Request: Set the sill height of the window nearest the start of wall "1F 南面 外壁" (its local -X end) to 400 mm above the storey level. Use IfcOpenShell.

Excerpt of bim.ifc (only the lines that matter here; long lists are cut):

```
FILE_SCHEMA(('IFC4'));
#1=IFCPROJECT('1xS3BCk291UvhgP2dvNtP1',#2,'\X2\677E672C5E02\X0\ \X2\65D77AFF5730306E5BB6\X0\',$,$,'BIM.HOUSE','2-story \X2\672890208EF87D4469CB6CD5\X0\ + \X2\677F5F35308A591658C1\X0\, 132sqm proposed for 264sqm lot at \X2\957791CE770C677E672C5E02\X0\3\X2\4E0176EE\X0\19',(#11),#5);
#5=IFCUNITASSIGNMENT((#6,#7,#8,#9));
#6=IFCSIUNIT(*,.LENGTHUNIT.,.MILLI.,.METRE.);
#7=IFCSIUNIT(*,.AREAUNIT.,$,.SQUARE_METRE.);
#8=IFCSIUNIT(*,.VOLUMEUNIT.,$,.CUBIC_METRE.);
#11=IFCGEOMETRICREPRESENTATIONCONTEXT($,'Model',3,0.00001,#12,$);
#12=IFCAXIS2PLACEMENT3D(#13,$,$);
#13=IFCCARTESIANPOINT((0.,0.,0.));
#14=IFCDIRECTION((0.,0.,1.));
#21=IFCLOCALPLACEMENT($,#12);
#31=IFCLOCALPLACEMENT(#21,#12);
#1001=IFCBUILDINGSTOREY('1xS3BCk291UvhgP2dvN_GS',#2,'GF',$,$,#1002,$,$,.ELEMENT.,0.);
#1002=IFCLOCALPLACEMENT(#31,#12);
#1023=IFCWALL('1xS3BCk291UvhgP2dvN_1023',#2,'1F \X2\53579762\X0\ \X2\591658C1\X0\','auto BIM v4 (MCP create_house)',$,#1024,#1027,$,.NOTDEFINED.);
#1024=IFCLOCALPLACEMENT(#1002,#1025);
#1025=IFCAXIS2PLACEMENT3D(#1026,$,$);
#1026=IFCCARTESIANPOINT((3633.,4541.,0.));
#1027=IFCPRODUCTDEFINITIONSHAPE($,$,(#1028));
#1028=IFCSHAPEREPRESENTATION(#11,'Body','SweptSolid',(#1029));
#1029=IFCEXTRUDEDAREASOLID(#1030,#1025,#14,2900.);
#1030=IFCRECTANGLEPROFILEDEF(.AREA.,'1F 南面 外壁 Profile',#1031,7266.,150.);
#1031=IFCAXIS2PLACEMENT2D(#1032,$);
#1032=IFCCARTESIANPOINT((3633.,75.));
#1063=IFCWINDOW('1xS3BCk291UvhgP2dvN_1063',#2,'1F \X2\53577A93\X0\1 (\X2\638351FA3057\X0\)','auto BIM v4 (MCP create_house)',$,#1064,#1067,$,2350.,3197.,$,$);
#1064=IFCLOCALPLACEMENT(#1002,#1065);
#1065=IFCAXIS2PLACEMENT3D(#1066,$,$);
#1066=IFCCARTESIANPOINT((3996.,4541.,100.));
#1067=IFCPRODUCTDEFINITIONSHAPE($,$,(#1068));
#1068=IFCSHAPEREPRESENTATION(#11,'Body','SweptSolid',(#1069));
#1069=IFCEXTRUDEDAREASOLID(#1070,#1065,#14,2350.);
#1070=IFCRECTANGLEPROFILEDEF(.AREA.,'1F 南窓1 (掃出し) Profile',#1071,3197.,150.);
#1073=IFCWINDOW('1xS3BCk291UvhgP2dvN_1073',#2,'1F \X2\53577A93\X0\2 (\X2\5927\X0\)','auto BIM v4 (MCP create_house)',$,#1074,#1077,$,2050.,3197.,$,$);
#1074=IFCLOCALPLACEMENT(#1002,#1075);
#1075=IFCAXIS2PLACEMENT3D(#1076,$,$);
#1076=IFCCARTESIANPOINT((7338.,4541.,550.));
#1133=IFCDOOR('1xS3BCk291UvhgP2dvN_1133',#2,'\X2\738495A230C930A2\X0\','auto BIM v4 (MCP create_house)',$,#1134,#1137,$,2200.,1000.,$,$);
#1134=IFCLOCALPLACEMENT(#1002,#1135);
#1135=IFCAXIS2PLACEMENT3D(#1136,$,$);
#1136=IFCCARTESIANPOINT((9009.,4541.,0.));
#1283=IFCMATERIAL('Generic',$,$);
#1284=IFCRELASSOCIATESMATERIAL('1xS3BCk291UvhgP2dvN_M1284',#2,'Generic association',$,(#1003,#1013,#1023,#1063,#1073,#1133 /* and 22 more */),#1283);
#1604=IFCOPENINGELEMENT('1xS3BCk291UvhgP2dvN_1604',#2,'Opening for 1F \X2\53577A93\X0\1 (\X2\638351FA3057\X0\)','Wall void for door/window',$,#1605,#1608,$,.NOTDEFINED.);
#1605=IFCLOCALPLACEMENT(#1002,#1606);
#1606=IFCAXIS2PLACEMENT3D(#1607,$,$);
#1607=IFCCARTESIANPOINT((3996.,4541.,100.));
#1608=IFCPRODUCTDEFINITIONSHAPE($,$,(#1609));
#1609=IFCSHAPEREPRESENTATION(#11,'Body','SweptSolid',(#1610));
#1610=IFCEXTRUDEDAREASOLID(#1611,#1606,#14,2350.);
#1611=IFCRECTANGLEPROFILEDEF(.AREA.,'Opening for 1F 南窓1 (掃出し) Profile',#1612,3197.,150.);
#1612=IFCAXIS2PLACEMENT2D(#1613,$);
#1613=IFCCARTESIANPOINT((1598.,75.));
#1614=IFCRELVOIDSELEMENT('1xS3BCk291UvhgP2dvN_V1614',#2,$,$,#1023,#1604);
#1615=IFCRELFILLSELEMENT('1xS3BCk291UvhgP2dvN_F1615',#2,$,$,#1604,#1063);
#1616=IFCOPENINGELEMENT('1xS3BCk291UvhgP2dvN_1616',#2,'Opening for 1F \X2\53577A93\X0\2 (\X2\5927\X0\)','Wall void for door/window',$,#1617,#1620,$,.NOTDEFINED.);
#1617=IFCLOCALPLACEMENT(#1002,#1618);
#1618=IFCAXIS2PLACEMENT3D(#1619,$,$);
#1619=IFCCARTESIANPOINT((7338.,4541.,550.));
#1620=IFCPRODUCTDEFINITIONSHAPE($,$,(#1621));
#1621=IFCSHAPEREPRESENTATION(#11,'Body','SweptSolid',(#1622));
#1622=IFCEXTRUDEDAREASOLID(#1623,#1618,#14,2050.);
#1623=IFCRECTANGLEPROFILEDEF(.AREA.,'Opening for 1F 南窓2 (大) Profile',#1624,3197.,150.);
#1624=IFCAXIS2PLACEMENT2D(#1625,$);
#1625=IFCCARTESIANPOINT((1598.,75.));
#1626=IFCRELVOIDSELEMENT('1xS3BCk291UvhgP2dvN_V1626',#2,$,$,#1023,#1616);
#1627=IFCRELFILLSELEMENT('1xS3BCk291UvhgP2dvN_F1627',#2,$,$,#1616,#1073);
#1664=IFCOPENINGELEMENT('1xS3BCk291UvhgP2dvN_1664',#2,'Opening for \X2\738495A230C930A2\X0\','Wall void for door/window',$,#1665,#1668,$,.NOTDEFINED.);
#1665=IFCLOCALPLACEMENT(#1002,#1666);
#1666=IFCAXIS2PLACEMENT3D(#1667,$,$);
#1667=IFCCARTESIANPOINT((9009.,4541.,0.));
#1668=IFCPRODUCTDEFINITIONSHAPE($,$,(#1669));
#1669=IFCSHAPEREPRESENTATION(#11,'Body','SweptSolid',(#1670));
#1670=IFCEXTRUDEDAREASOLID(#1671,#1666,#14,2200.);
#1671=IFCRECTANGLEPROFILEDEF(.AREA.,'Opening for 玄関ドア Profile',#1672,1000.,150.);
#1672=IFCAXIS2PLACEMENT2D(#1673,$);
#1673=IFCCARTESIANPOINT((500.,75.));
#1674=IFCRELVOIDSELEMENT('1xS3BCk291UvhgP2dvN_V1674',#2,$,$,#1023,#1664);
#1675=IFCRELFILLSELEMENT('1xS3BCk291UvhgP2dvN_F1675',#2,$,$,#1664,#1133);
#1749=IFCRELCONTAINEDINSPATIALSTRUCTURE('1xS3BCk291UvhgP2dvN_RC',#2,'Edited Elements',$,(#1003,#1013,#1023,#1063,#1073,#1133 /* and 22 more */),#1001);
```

```python
import numpy as np
import ifcopenshell
import ifcopenshell.api.geometry
import ifcopenshell.geom
import ifcopenshell.util.element
import ifcopenshell.util.placement
import ifcopenshell.util.shape
import ifcopenshell.util.unit

model = ifcopenshell.open("bim.ifc")
unit_scale = ifcopenshell.util.unit.calculate_unit_scale(model)

window = model.by_guid("1xS3BCk291UvhgP2dvN_1063")
opening = window.FillsVoids[0].RelatingOpeningElement
storey = ifcopenshell.util.element.get_container(window, ifc_class="IfcBuildingStorey")
level = ifcopenshell.util.placement.get_local_placement(storey.ObjectPlacement)[2, 3]

# The opening's origin need not be at the sill, so measure its lowest point.
shape = ifcopenshell.geom.create_shape(ifcopenshell.geom.settings(), opening)
bottom = ifcopenshell.util.shape.get_shape_bottom_elevation(shape, shape.geometry) / unit_scale
dz = level + 0.4 / unit_scale - bottom

shift = np.array([0.0, 0.0, dz])
# The window is not placed relative to its opening, so move both.
for product in (opening, window):
    matrix = ifcopenshell.util.placement.get_local_placement(product.ObjectPlacement)
    matrix[:3, 3] += shift
    ifcopenshell.api.geometry.edit_object_placement(model, product=product, matrix=matrix, is_si=False)

print(f"moved by {dz * unit_scale:+.3f} m")

model.write("bim_v2.ifc")
```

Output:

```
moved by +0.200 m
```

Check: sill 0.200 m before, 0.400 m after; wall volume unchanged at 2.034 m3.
